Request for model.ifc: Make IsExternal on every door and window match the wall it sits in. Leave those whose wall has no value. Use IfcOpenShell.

First a look at what the model holds.

```python
import ifcopenshell
import ifcopenshell.util.element

model = ifcopenshell.open("model.ifc")
print(model.schema)
seen = {}
for e in model.by_type("IfcDoor") + model.by_type("IfcWindow"):
    if not e.FillsVoids:
        continue
    host = e.FillsVoids[0].RelatingOpeningElement.VoidsElements[0].RelatingBuildingElement
    own = ifcopenshell.util.element.get_pset(e, f"Pset_{e.is_a()[3:].removesuffix('StandardCase')}Common", "IsExternal")
    wall = ifcopenshell.util.element.get_pset(host, "Pset_WallCommon", "IsExternal")
    seen[e.is_a(), own, wall] = seen.get((e.is_a(), own, wall), 0) + 1
for (cls, own, wall), count in sorted(seen.items(), key=str):
    print(count, cls, "IsExternal:", own, "| host wall:", wall)
```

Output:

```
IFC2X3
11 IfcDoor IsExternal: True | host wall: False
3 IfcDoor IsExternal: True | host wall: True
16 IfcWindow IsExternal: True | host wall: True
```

```python
import ifcopenshell
import ifcopenshell.api.pset
import ifcopenshell.util.element

model = ifcopenshell.open("model.ifc")

count = 0
for ifc_class, pset_name in (("IfcDoor", "Pset_DoorCommon"), ("IfcWindow", "Pset_WindowCommon")):
    for e in model.by_type(ifc_class):
        if not e.FillsVoids:
            continue
        host = e.FillsVoids[0].RelatingOpeningElement.VoidsElements[0].RelatingBuildingElement
        external = ifcopenshell.util.element.get_pset(host, "Pset_WallCommon", "IsExternal")
        if external is None or ifcopenshell.util.element.get_pset(e, pset_name, "IsExternal") == external:
            continue
        pset = ifcopenshell.api.pset.add_pset(model, product=e, name=pset_name)
        ifcopenshell.api.pset.edit_pset(model, pset=pset, properties={"IsExternal": external})
        count += 1

print(count, "updated")

model.write("model_edited.ifc")
```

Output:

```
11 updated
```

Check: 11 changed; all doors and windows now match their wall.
